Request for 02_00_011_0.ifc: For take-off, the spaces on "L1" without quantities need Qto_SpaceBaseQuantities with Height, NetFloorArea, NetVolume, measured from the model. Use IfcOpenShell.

First a look at what the model holds.

```python
import ifcopenshell
import ifcopenshell.util.element
import ifcopenshell.util.unit

model = ifcopenshell.open("02_00_011_0.ifc")
print(model.schema)
for unit_type in ("LENGTHUNIT", "AREAUNIT", "VOLUMEUNIT"):
    print(unit_type, ifcopenshell.util.unit.calculate_unit_scale(model, unit_type))
storey = next(s for s in model.by_type("IfcBuildingStorey") if s.Name == "L1")
spaces = [e for e in ifcopenshell.util.element.get_decomposition(storey) if e.is_a("IfcSpace")]
for e in sorted(spaces, key=lambda e: e.id()):
    print(e.id(), e.is_a(), e.Name, list(ifcopenshell.util.element.get_psets(e, qtos_only=True)), sep=" | ")
```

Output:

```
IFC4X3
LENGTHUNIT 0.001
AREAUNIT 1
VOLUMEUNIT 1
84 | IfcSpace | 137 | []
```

```python
import ifcopenshell
import ifcopenshell.api.pset
import ifcopenshell.geom
import ifcopenshell.util.element
import ifcopenshell.util.shape
import ifcopenshell.util.unit

model = ifcopenshell.open("02_00_011_0.ifc")
unit_scale = ifcopenshell.util.unit.calculate_unit_scale(model)
area_scale = ifcopenshell.util.unit.calculate_unit_scale(model, "AREAUNIT")
volume_scale = ifcopenshell.util.unit.calculate_unit_scale(model, "VOLUMEUNIT")
settings = ifcopenshell.geom.settings()

storey = next(s for s in model.by_type("IfcBuildingStorey") if s.Name == "L1")
spaces = [e for e in ifcopenshell.util.element.get_decomposition(storey) if e.is_a("IfcSpace")]

for e in sorted(spaces, key=lambda e: e.id()):
    if ifcopenshell.util.element.get_psets(e, qtos_only=True, should_inherit=False):
        continue
    # Geometry comes back in metres, in the element's own axes.
    shape = ifcopenshell.geom.create_shape(settings, e)
    values = {
        "Height": ifcopenshell.util.shape.get_z(shape.geometry) / unit_scale,
        "NetFloorArea": ifcopenshell.util.shape.get_footprint_area(shape.geometry) / area_scale,
        "NetVolume": ifcopenshell.util.shape.get_volume(shape.geometry) / volume_scale,
    }
    qto = ifcopenshell.api.pset.add_qto(model, product=e, name="Qto_SpaceBaseQuantities")
    ifcopenshell.api.pset.edit_qto(model, qto=qto, properties=values)
    print(e.id(), {k: round(v, 3) for k, v in values.items()})

model.write("02_00_011_0_rev.ifc")
```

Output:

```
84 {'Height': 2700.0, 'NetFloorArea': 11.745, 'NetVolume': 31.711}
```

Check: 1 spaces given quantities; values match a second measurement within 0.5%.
